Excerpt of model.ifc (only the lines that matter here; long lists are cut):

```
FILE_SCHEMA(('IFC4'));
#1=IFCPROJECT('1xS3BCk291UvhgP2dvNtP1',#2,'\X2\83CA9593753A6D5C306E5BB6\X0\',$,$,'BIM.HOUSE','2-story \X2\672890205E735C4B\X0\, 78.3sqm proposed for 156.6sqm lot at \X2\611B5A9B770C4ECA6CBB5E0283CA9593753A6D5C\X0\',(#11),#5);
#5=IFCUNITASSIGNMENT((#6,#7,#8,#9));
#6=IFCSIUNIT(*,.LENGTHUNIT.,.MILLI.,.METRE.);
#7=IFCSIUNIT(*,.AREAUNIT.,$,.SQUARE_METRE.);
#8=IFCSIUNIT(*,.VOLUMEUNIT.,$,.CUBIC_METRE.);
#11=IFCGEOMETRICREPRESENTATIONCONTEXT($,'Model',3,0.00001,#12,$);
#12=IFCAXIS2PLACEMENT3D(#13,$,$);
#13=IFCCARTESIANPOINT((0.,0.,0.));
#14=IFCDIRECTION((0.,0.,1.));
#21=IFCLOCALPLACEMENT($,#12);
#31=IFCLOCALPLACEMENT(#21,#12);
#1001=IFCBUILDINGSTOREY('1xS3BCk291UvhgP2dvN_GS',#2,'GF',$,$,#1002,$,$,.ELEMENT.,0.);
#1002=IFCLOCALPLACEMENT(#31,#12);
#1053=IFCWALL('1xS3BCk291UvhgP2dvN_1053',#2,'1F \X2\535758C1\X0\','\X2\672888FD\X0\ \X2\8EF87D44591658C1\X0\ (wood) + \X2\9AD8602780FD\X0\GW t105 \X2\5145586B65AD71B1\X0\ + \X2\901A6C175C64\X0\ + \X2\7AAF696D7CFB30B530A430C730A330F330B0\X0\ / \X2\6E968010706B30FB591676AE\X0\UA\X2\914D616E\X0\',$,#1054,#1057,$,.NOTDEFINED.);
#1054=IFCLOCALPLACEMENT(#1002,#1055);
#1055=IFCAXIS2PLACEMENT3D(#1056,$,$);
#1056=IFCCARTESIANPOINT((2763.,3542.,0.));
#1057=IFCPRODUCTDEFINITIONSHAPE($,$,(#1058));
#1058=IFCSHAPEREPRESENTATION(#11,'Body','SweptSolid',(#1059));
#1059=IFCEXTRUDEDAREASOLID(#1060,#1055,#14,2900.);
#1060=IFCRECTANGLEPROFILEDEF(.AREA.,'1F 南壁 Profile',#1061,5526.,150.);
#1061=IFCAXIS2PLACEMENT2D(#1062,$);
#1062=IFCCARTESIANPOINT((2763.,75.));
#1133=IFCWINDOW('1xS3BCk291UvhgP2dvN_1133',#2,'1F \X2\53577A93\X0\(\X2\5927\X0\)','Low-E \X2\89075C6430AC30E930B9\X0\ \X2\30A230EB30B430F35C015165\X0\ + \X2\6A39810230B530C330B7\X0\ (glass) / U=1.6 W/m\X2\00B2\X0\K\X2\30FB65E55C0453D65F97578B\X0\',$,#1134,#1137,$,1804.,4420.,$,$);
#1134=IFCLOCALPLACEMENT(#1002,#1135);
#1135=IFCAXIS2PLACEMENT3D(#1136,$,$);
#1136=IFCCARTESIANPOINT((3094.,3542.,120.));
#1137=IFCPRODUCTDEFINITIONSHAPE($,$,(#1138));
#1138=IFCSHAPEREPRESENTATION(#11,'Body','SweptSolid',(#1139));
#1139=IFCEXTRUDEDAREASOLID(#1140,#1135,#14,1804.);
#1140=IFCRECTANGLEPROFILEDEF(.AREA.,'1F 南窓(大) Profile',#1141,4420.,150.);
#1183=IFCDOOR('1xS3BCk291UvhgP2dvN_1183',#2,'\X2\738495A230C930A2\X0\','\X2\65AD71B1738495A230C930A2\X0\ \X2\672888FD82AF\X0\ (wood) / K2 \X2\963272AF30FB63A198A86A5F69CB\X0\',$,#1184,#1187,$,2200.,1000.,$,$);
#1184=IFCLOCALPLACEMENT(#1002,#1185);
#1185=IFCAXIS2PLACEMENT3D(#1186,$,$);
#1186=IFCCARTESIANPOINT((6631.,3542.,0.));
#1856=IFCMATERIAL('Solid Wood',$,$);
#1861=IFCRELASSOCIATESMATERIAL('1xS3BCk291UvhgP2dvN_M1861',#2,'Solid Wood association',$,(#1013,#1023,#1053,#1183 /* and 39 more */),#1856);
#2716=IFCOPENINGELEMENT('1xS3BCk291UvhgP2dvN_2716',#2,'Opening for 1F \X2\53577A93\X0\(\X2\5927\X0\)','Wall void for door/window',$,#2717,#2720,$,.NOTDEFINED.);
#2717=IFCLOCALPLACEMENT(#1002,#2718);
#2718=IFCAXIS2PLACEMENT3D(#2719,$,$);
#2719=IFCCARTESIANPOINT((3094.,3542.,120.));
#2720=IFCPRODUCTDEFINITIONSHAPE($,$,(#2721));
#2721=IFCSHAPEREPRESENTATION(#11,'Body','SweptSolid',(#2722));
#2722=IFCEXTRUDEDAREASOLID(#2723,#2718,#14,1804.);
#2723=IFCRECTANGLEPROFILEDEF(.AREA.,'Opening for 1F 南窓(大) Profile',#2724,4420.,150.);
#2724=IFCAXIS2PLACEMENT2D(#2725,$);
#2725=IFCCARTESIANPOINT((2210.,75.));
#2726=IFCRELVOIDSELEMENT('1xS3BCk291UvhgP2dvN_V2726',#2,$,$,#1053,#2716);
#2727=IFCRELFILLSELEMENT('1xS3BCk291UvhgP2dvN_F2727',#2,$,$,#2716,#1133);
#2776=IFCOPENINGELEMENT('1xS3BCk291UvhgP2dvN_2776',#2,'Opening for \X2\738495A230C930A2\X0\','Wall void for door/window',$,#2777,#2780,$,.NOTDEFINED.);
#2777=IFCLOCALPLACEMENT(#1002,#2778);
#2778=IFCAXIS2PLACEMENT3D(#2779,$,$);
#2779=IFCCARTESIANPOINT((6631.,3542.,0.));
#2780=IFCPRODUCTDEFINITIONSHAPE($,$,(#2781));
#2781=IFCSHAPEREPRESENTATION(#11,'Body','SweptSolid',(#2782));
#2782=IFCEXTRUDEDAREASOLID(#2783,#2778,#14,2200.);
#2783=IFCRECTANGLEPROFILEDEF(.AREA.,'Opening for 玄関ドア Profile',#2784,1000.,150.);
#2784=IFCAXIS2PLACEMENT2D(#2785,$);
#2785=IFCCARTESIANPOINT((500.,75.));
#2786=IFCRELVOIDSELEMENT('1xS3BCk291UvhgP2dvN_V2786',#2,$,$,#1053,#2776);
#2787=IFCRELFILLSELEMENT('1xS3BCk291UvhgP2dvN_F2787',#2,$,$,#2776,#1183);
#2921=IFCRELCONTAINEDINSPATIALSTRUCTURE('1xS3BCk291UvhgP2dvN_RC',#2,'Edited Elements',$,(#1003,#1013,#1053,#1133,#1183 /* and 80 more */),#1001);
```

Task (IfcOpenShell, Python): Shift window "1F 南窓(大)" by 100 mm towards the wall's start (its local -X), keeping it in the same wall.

```python
import ifcopenshell
import ifcopenshell.api.geometry
import ifcopenshell.util.placement
import ifcopenshell.util.unit

model = ifcopenshell.open("model.ifc")
unit_scale = ifcopenshell.util.unit.calculate_unit_scale(model)

window = model.by_guid("1xS3BCk291UvhgP2dvN_1133")
opening = window.FillsVoids[0].RelatingOpeningElement
wall = opening.VoidsElements[0].RelatingBuildingElement

wall_matrix = ifcopenshell.util.placement.get_local_placement(wall.ObjectPlacement)
shift = wall_matrix[:3, 0] * -0.1 / unit_scale
before = ifcopenshell.util.placement.get_local_placement(window.ObjectPlacement)[:3, 3].copy()

# The window is not placed relative to its opening, so move both.
for product in (opening, window):
    matrix = ifcopenshell.util.placement.get_local_placement(product.ObjectPlacement)
    matrix[:3, 3] += shift
    ifcopenshell.api.geometry.edit_object_placement(model, product=product, matrix=matrix, is_si=False)

after = ifcopenshell.util.placement.get_local_placement(window.ObjectPlacement)[:3, 3]
print("window moved by", (after - before).round(3) + 0.0)

model.write("model-out.ifc")
```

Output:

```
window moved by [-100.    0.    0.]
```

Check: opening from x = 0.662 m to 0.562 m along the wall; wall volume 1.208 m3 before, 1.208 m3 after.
